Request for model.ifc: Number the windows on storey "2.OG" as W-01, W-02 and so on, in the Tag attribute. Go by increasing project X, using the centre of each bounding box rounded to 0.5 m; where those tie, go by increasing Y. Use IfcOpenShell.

First a look at what the model holds.

```python
import ifcopenshell
import ifcopenshell.util.element
import ifcopenshell.util.placement

model = ifcopenshell.open("model.ifc")
print(model.schema)
storey = next(s for s in model.by_type("IfcBuildingStorey") if s.Name == "2.OG")
windows = [e for e in ifcopenshell.util.element.get_decomposition(storey) if e.is_a("IfcWindow")]
for e in sorted(windows, key=lambda e: e.id()):
    origin = ifcopenshell.util.placement.get_local_placement(e.ObjectPlacement)[:3, 3]
    print(e.id(), e.Tag, e.Name, origin.round(2) + 0.0, sep=" | ")
```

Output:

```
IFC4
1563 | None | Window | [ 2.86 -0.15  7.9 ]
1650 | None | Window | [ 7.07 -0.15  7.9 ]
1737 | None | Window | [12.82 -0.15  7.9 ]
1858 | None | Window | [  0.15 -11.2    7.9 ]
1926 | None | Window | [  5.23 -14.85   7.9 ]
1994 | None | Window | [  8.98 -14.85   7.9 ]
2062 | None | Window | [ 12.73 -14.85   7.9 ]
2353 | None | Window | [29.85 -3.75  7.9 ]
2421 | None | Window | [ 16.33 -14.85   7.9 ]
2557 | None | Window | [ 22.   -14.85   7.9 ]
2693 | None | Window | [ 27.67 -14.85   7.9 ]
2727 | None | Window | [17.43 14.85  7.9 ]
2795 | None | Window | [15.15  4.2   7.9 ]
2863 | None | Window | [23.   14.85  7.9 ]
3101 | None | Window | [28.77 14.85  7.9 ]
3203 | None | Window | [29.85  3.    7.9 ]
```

```python
import ifcopenshell
import ifcopenshell.geom
import ifcopenshell.util.element
import ifcopenshell.util.shape

model = ifcopenshell.open("model.ifc")
settings = ifcopenshell.geom.settings()
settings.set("use-world-coords", True)


def centre(element):
    shape = ifcopenshell.geom.create_shape(settings, element)
    return ifcopenshell.util.shape.get_bbox_centroid(shape.geometry)


storey = next(s for s in model.by_type("IfcBuildingStorey") if s.Name == "2.OG")
windows = [e for e in ifcopenshell.util.element.get_decomposition(storey) if e.is_a("IfcWindow")]

# Insertion points can sit at a corner or the storey origin, so sort by the geometry (in metres).
centres = {e: centre(e) for e in windows}
windows.sort(key=lambda e: (round(centres[e][0] / 0.5), centres[e][1]))

for i, e in enumerate(windows, start=1):
    number = f"W-{i:02d}"
    e.Tag = number
    print(e.id(), number)

model.write("model_rev.ifc")
```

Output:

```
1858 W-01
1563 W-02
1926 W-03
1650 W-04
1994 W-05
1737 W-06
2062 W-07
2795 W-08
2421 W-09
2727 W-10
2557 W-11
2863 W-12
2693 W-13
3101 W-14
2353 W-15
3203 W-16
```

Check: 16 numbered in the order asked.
